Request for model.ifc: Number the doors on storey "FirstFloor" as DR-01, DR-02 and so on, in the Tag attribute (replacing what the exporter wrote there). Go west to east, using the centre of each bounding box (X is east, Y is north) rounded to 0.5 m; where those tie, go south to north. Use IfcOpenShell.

First a look at what the model holds.

```python
import ifcopenshell
import ifcopenshell.util.element
import ifcopenshell.util.placement

model = ifcopenshell.open("model.ifc")
print(model.schema)
storey = next(s for s in model.by_type("IfcBuildingStorey") if s.Name == "FirstFloor")
doors = [e for e in ifcopenshell.util.element.get_decomposition(storey) if e.is_a("IfcDoor")]
for e in sorted(doors, key=lambda e: e.id()):
    origin = ifcopenshell.util.placement.get_local_placement(e.ObjectPlacement)[:3, 3]
    print(e.id(), e.Tag, e.Name, origin.round(2) + 0.0, sep=" | ")
```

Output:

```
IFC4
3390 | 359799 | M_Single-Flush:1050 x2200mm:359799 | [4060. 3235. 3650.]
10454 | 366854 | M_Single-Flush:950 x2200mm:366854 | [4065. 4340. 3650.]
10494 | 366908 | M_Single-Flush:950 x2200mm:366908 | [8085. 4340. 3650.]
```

```python
import ifcopenshell
import ifcopenshell.geom
import ifcopenshell.util.element
import ifcopenshell.util.shape

model = ifcopenshell.open("model.ifc")
settings = ifcopenshell.geom.settings()
settings.set("use-world-coords", True)


def centre(element):
    shape = ifcopenshell.geom.create_shape(settings, element)
    return ifcopenshell.util.shape.get_bbox_centroid(shape.geometry)


storey = next(s for s in model.by_type("IfcBuildingStorey") if s.Name == "FirstFloor")
doors = [e for e in ifcopenshell.util.element.get_decomposition(storey) if e.is_a("IfcDoor")]

# Insertion points can sit at a corner or the storey origin, so sort by the geometry (in metres).
centres = {e: centre(e) for e in doors}
doors.sort(key=lambda e: (round(centres[e][0] / 0.5), centres[e][1]))

for i, e in enumerate(doors, start=1):
    number = f"DR-{i:02d}"
    e.Tag = number
    print(e.id(), number)

model.write("model_updated.ifc")
```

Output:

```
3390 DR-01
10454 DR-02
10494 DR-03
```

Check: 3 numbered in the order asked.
